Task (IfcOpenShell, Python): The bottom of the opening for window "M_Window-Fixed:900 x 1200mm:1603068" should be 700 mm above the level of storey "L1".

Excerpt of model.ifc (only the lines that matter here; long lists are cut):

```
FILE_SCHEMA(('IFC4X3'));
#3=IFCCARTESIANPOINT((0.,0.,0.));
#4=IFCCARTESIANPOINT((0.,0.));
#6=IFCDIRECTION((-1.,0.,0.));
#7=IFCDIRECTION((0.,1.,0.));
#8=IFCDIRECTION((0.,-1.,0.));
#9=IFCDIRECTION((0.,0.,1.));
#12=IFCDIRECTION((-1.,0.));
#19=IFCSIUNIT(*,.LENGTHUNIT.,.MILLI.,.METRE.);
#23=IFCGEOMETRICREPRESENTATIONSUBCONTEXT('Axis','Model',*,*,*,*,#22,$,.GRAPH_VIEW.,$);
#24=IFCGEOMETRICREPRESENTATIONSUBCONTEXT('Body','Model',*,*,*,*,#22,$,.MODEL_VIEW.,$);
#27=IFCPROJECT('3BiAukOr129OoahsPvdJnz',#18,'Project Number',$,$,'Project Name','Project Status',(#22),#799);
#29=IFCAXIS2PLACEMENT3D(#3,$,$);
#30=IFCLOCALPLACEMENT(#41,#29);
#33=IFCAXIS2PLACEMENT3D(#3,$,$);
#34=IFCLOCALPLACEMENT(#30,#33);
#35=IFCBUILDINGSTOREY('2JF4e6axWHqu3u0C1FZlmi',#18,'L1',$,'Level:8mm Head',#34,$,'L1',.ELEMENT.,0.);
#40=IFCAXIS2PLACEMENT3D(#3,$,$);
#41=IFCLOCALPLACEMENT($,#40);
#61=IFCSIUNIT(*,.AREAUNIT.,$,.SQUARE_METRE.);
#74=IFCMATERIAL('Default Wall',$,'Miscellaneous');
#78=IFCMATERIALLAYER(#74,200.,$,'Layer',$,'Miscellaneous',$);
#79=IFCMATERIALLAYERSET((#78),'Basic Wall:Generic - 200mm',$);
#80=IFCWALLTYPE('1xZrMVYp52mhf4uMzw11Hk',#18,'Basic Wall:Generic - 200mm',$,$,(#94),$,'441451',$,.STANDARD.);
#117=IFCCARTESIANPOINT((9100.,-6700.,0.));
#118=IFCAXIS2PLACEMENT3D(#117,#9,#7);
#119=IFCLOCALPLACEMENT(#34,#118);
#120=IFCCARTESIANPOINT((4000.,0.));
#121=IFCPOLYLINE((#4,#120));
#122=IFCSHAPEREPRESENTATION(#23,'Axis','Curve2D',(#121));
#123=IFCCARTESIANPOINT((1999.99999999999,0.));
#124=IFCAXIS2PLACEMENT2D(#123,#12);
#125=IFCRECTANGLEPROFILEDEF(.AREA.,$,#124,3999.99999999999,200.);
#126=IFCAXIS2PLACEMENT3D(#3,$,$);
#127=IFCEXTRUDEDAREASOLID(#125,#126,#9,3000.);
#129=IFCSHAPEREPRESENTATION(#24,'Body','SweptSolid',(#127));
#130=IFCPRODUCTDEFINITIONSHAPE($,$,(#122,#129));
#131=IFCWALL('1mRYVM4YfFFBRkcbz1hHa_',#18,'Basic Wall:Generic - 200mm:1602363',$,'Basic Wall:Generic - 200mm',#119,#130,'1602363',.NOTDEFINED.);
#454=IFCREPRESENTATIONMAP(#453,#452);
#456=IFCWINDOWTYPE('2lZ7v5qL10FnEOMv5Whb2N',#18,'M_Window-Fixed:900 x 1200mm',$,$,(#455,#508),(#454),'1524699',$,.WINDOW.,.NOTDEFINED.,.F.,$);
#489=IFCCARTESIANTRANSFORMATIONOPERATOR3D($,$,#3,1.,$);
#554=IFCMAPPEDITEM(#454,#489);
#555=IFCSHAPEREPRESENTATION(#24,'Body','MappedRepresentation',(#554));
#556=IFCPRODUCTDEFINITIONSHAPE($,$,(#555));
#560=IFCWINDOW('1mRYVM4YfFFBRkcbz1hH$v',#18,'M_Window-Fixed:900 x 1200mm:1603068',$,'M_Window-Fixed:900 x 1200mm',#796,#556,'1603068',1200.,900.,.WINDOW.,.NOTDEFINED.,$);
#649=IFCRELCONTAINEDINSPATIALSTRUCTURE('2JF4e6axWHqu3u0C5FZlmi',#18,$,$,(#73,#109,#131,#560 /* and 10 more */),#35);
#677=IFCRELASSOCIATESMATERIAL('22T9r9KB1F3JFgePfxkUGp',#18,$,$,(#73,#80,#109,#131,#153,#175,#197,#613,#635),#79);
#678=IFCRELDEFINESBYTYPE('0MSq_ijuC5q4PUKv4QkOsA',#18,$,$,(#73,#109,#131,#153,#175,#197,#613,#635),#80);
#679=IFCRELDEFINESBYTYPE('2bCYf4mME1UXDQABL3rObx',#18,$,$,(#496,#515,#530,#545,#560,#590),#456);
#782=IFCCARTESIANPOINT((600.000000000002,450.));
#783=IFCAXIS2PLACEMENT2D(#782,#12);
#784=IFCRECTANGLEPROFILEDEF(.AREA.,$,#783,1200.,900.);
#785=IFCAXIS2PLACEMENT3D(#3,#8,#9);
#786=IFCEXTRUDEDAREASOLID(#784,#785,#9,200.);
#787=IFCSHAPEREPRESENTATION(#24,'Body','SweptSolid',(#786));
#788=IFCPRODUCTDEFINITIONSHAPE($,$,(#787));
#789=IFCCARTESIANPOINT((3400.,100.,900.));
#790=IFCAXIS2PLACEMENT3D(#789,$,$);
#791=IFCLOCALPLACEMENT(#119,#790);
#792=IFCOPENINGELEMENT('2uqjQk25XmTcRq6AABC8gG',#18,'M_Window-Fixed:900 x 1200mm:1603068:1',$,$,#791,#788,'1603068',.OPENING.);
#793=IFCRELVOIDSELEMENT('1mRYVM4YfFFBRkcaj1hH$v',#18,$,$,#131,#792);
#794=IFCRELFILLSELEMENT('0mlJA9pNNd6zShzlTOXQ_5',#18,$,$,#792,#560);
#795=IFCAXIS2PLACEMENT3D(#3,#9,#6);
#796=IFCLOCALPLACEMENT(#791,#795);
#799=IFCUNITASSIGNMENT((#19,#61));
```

```python
import numpy as np
import ifcopenshell
import ifcopenshell.api.geometry
import ifcopenshell.geom
import ifcopenshell.util.element
import ifcopenshell.util.placement
import ifcopenshell.util.shape
import ifcopenshell.util.unit

model = ifcopenshell.open("model.ifc")
unit_scale = ifcopenshell.util.unit.calculate_unit_scale(model)

window = model.by_guid("1mRYVM4YfFFBRkcbz1hH$v")
opening = window.FillsVoids[0].RelatingOpeningElement
storey = ifcopenshell.util.element.get_container(window, ifc_class="IfcBuildingStorey")
level = ifcopenshell.util.placement.get_local_placement(storey.ObjectPlacement)[2, 3]

# The opening's origin need not be at the sill, so measure its lowest point.
shape = ifcopenshell.geom.create_shape(ifcopenshell.geom.settings(), opening)
bottom = ifcopenshell.util.shape.get_shape_bottom_elevation(shape, shape.geometry) / unit_scale
dz = level + 700.0 - bottom

shift = np.array([0.0, 0.0, dz])
# The window is placed relative to its opening, so it follows when the opening moves.
matrix = ifcopenshell.util.placement.get_local_placement(opening.ObjectPlacement)
matrix[:3, 3] += shift
ifcopenshell.api.geometry.edit_object_placement(
    model, product=opening, matrix=matrix, is_si=False, should_transform_children=True
)

print(f"moved by {dz * unit_scale:+.3f} m")

model.write("model_updated.ifc")
```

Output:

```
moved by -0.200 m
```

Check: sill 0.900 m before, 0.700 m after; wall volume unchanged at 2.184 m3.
